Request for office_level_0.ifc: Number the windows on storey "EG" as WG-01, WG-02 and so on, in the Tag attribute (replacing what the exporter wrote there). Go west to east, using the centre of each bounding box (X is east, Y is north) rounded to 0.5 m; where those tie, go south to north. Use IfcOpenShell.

First a look at what the model holds.

```python
import ifcopenshell
import ifcopenshell.util.element
import ifcopenshell.util.placement

model = ifcopenshell.open("office_level_0.ifc")
print(model.schema)
storey = next(s for s in model.by_type("IfcBuildingStorey") if s.Name == "EG")
windows = [e for e in ifcopenshell.util.element.get_decomposition(storey) if e.is_a("IfcWindow")]
for e in sorted(windows, key=lambda e: e.id()):
    origin = ifcopenshell.util.placement.get_local_placement(e.ObjectPlacement)[:3, 3]
    print(e.id(), e.Tag, e.Name, origin.round(2) + 0.0, sep=" | ")
```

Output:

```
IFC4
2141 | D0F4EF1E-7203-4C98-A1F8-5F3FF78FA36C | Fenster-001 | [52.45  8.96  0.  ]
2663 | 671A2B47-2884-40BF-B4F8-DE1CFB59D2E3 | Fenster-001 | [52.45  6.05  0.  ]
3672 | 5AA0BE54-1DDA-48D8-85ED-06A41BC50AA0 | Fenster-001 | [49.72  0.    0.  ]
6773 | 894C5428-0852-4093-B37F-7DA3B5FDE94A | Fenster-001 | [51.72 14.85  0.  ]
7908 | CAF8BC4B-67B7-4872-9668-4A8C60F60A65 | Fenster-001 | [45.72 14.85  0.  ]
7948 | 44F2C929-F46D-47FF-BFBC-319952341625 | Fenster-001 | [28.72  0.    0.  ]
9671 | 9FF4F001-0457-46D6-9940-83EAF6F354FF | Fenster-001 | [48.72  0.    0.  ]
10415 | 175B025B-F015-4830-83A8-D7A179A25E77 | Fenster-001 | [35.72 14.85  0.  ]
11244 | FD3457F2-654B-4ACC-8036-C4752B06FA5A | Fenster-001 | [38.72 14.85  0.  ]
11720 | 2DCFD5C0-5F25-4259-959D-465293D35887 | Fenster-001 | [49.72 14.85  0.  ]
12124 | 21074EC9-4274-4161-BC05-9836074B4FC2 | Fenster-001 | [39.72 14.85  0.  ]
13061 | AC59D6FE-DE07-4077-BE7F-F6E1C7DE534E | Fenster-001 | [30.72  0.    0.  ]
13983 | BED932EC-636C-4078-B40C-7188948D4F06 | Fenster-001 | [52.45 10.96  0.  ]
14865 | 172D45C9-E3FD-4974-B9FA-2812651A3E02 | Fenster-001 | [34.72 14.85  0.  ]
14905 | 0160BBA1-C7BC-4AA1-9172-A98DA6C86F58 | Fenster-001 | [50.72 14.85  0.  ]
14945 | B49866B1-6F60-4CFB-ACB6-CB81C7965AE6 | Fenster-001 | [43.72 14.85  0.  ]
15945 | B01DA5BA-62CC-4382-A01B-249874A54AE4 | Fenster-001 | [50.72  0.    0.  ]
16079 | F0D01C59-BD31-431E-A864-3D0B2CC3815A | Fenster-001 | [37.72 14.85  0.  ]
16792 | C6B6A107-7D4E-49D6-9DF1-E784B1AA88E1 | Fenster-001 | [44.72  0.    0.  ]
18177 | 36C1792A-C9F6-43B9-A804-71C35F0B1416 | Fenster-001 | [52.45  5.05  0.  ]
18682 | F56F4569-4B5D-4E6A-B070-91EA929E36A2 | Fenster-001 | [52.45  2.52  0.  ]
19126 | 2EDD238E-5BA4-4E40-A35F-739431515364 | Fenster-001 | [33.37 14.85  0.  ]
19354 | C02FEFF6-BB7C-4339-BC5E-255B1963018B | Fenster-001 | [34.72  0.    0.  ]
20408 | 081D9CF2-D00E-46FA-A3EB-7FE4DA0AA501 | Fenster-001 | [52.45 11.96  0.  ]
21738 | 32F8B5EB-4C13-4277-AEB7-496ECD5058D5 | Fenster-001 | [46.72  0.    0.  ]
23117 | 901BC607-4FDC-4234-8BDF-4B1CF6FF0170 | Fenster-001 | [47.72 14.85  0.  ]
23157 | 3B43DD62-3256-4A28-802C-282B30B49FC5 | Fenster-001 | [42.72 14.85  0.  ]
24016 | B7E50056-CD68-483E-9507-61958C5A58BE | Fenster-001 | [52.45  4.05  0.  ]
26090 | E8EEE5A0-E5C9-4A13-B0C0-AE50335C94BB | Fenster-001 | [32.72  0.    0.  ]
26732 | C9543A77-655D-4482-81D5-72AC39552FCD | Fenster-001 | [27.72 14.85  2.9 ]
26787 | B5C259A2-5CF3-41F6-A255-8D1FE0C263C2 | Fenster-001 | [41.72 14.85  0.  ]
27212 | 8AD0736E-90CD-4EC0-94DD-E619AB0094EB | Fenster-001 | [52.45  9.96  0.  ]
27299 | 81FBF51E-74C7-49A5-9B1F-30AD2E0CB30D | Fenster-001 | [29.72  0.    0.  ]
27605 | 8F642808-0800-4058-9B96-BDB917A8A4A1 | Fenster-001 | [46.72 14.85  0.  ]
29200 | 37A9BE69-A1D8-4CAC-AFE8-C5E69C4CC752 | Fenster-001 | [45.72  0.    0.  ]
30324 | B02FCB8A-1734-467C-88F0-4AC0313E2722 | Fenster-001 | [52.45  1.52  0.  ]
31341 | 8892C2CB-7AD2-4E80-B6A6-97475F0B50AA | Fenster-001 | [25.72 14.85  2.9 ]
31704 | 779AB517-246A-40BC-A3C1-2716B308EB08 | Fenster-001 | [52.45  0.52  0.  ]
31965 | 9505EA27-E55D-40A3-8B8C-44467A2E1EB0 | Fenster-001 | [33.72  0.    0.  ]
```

```python
import ifcopenshell
import ifcopenshell.geom
import ifcopenshell.util.element
import ifcopenshell.util.shape

model = ifcopenshell.open("office_level_0.ifc")
settings = ifcopenshell.geom.settings()
settings.set("use-world-coords", True)


def centre(element):
    shape = ifcopenshell.geom.create_shape(settings, element)
    return ifcopenshell.util.shape.get_bbox_centroid(shape.geometry)


storey = next(s for s in model.by_type("IfcBuildingStorey") if s.Name == "EG")
windows = [e for e in ifcopenshell.util.element.get_decomposition(storey) if e.is_a("IfcWindow")]

# Insertion points can sit at a corner or the storey origin, so sort by the geometry (in metres).
centres = {e: centre(e) for e in windows}
windows.sort(key=lambda e: (round(centres[e][0] / 0.5), centres[e][1]))

for i, e in enumerate(windows, start=1):
    number = f"WG-{i:02d}"
    e.Tag = number
    print(e.id(), number)

model.write("office_level_0_updated.ifc")
```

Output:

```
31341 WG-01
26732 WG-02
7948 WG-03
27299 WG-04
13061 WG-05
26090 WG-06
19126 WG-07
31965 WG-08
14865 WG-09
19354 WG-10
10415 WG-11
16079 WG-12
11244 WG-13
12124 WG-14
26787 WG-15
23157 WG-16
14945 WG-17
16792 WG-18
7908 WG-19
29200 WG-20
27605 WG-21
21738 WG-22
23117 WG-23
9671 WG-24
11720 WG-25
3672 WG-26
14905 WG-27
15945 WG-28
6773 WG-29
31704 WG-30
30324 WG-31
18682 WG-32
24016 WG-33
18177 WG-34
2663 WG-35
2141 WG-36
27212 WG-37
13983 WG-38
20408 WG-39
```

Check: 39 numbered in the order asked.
